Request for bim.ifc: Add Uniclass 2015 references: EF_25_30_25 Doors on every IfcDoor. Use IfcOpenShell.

First a look at what the model holds.

```python
import ifcopenshell

model = ifcopenshell.open("bim.ifc")
print(model.schema)
print("classifications:", [c.Name for c in model.by_type("IfcClassification")])
for ifc_class in ("IfcDoor", "IfcRoof", "IfcStair", "IfcWall", "IfcWindow"):
    print(ifc_class, len(model.by_type(ifc_class)))
```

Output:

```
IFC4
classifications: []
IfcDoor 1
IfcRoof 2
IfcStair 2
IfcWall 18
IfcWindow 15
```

```python
import ifcopenshell
import ifcopenshell.api.classification

model = ifcopenshell.open("bim.ifc")

system = ifcopenshell.api.classification.add_classification(model, classification="Uniclass 2015")

codes = {
    "IfcDoor": ("EF_25_30_25", "Doors"),
}
for ifc_class, (code, name) in codes.items():
    products = model.by_type(ifc_class)
    ifcopenshell.api.classification.add_reference(
        model, products=products, classification=system, identification=code, name=name
    )
    print(code, len(products))

model.write("bim_edited.ifc")
```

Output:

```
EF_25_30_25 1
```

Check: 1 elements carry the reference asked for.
